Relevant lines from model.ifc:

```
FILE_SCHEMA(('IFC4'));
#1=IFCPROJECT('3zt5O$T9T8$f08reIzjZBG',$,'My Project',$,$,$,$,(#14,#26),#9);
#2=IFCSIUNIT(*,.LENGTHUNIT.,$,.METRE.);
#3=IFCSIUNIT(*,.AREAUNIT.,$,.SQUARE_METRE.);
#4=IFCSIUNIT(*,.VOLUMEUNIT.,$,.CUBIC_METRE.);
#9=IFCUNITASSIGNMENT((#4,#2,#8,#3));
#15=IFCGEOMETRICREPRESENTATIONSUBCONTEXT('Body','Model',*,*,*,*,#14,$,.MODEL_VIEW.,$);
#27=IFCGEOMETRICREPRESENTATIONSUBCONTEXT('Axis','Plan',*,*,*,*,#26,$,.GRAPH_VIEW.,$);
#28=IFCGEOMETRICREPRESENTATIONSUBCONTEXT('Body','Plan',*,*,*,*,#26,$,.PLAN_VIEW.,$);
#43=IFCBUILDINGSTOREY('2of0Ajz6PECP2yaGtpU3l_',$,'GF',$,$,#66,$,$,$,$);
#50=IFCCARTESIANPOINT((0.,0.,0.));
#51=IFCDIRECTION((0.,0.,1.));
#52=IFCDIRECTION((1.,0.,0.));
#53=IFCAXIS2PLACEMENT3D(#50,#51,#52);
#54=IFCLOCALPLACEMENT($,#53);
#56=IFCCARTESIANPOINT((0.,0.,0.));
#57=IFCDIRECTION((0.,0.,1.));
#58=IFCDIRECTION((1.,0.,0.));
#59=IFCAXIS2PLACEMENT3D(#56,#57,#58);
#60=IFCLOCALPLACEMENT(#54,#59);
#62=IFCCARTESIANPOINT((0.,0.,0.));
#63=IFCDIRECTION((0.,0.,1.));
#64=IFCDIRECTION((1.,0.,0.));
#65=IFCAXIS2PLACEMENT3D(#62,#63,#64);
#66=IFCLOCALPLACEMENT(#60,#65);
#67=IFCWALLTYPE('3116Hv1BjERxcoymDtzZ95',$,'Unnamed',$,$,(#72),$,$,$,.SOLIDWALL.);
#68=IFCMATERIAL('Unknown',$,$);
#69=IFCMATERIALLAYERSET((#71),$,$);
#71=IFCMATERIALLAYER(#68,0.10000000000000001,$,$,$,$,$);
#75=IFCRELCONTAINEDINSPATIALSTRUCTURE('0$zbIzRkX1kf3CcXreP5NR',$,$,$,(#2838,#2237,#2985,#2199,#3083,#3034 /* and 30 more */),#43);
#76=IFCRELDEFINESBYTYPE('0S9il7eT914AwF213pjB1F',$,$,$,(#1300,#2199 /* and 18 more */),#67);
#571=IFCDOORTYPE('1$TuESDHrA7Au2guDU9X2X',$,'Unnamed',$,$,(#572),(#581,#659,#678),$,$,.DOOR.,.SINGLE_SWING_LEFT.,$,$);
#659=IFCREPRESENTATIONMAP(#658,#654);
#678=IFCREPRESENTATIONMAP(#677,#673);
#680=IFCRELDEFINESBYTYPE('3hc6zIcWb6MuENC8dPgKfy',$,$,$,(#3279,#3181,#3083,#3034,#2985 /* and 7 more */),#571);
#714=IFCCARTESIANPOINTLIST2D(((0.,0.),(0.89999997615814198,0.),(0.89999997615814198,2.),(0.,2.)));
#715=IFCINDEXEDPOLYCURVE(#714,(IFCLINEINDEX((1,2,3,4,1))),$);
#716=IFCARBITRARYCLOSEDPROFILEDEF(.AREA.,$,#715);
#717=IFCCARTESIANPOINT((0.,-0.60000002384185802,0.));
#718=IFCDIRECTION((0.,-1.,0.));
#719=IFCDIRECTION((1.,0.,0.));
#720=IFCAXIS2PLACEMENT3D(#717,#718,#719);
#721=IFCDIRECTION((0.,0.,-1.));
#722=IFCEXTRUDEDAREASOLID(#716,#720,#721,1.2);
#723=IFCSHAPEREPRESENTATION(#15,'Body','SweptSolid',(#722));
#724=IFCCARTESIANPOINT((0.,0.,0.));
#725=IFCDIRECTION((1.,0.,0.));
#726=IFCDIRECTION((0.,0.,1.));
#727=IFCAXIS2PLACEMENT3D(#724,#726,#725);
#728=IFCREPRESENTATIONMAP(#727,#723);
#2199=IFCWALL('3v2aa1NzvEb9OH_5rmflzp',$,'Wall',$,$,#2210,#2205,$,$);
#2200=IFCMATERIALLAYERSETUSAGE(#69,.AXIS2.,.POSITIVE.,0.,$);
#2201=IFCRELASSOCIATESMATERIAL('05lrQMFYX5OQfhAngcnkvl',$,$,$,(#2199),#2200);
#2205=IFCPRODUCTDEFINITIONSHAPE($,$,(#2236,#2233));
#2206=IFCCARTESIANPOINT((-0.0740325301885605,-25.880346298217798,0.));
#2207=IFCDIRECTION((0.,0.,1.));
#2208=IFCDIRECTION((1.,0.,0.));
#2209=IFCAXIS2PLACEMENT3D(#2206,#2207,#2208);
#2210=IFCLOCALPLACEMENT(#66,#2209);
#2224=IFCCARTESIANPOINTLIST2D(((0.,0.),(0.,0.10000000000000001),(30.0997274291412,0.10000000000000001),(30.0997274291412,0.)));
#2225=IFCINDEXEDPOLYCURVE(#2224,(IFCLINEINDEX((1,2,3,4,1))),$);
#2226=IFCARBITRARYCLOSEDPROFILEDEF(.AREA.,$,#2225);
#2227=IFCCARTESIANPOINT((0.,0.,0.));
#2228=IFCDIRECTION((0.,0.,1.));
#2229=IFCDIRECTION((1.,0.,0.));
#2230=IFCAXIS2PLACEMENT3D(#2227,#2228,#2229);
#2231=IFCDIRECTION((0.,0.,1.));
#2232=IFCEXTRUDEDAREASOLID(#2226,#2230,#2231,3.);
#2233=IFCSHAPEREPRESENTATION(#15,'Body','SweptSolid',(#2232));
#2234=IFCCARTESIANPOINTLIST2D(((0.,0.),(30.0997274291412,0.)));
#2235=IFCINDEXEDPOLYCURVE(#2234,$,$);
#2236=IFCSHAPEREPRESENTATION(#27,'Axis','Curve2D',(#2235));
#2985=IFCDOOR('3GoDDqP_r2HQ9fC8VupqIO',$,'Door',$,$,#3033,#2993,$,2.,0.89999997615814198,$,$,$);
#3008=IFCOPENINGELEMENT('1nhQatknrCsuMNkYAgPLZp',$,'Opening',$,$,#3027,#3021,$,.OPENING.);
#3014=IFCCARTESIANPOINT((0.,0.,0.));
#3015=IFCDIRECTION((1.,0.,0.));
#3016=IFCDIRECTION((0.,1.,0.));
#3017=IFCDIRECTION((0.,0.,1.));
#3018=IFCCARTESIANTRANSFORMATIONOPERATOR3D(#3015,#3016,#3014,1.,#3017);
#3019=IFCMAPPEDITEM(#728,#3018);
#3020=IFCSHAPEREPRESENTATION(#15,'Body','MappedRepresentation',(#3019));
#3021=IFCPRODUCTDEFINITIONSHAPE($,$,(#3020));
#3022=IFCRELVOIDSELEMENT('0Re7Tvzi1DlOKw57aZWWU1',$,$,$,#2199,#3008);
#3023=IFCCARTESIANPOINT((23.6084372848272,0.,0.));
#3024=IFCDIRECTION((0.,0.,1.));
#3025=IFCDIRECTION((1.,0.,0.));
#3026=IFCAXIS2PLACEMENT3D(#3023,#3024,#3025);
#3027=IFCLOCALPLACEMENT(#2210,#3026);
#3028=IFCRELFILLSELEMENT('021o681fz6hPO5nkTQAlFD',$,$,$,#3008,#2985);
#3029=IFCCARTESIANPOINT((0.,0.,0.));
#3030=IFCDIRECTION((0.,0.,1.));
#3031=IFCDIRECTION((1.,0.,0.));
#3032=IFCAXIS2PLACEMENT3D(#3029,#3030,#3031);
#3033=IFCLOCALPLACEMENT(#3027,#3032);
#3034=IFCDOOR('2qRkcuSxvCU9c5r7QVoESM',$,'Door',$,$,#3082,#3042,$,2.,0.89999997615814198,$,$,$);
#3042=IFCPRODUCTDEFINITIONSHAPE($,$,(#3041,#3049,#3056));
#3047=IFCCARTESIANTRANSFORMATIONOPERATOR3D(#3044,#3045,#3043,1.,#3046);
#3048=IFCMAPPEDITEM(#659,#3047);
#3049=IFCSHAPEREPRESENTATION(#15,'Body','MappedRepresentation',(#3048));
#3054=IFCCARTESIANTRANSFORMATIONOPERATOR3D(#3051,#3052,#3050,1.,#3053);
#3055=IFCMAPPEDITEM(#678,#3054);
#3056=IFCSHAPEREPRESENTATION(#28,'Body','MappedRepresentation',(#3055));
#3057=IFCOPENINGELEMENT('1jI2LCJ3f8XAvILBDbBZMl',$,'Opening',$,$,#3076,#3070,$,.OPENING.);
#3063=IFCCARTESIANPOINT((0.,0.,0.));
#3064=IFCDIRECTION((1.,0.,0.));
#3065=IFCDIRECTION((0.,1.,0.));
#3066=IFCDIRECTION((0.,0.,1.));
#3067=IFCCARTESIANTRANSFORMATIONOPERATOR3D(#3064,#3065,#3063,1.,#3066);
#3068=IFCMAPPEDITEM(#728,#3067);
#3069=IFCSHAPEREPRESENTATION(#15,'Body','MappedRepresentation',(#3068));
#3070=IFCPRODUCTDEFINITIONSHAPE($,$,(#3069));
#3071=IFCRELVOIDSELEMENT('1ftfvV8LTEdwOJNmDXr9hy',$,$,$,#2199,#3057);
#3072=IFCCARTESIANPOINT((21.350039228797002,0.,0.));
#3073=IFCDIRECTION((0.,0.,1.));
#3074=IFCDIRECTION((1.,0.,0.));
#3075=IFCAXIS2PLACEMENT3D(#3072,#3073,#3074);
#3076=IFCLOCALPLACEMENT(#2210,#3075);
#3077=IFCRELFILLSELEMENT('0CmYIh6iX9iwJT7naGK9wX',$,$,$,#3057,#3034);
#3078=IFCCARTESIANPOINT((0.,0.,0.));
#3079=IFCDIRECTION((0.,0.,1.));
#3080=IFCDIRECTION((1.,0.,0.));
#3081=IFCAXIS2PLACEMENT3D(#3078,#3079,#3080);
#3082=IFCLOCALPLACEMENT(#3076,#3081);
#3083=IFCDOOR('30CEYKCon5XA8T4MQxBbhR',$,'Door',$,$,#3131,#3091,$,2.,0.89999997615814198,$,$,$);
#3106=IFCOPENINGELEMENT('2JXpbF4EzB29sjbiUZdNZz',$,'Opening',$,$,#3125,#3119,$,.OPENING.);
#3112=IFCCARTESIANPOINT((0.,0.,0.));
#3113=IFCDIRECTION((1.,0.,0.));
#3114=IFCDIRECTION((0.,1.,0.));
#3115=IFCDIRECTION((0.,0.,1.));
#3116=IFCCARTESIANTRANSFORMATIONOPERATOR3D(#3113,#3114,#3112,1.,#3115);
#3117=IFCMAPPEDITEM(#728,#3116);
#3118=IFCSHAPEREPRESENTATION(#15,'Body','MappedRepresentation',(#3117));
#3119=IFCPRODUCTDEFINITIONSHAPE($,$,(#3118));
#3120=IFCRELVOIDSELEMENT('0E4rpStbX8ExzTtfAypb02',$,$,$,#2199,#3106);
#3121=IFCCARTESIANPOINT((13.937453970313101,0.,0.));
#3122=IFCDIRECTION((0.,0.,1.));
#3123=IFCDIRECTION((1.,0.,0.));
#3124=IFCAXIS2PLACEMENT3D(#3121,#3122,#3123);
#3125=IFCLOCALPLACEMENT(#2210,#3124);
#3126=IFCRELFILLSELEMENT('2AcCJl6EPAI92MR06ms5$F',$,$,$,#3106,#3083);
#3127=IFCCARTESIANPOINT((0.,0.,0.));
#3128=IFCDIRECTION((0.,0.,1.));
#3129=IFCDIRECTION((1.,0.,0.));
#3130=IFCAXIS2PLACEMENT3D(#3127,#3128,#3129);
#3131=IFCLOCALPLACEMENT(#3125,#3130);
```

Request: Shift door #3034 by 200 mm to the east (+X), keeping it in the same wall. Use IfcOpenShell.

```python
import ifcopenshell
import ifcopenshell.api.geometry
import ifcopenshell.util.placement
import ifcopenshell.util.unit

model = ifcopenshell.open("model.ifc")
unit_scale = ifcopenshell.util.unit.calculate_unit_scale(model)

door = model.by_id(3034)
opening = door.FillsVoids[0].RelatingOpeningElement
wall = opening.VoidsElements[0].RelatingBuildingElement

wall_matrix = ifcopenshell.util.placement.get_local_placement(wall.ObjectPlacement)
shift = wall_matrix[:3, 0] * 0.2 / unit_scale
before = ifcopenshell.util.placement.get_local_placement(door.ObjectPlacement)[:3, 3].copy()

# The door is placed relative to its opening, so it follows when the opening moves.
matrix = ifcopenshell.util.placement.get_local_placement(opening.ObjectPlacement)
matrix[:3, 3] += shift
ifcopenshell.api.geometry.edit_object_placement(
    model, product=opening, matrix=matrix, is_si=False, should_transform_children=True
)

after = ifcopenshell.util.placement.get_local_placement(door.ObjectPlacement)[:3, 3]
print("door moved by", (after - before).round(3) + 0.0)

model.write("model_updated.ifc")
```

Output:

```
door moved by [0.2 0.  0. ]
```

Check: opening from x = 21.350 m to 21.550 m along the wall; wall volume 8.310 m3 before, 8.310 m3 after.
